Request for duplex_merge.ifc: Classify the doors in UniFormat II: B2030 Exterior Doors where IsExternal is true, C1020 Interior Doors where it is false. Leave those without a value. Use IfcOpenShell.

First a look at what the model holds.

```python
import ifcopenshell
import ifcopenshell.util.element

model = ifcopenshell.open("duplex_merge.ifc")
print(model.schema)
print("classifications:", [c.Name for c in model.by_type("IfcClassification")])
values = [ifcopenshell.util.element.get_pset(e, "Pset_DoorCommon", "IsExternal") for e in model.by_type("IfcDoor")]
for value in (True, False, None):
    print("IsExternal", value, values.count(value))
```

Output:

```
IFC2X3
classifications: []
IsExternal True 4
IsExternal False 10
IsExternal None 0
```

```python
import ifcopenshell
import ifcopenshell.api.classification
import ifcopenshell.util.element

model = ifcopenshell.open("duplex_merge.ifc")

# IFC2X3 requires Source and Edition and has no link from the project to the system.
system = model.create_entity("IfcClassification", Source="ASTM", Edition="E1557", Name="UniFormat II")

doors = model.by_type("IfcDoor")
external = {e: ifcopenshell.util.element.get_pset(e, "Pset_DoorCommon", "IsExternal") for e in doors}
for flag, code, name in ((True, "B2030", "Exterior Doors"), (False, "C1020", "Interior Doors")):
    products = [e for e in doors if external[e] is flag]
    ifcopenshell.api.classification.add_reference(
        model, products=products, classification=system, identification=code, name=name
    )
    print(code, len(products))

model.write("duplex_merge_edited.ifc")
```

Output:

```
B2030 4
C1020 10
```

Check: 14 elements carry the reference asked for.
